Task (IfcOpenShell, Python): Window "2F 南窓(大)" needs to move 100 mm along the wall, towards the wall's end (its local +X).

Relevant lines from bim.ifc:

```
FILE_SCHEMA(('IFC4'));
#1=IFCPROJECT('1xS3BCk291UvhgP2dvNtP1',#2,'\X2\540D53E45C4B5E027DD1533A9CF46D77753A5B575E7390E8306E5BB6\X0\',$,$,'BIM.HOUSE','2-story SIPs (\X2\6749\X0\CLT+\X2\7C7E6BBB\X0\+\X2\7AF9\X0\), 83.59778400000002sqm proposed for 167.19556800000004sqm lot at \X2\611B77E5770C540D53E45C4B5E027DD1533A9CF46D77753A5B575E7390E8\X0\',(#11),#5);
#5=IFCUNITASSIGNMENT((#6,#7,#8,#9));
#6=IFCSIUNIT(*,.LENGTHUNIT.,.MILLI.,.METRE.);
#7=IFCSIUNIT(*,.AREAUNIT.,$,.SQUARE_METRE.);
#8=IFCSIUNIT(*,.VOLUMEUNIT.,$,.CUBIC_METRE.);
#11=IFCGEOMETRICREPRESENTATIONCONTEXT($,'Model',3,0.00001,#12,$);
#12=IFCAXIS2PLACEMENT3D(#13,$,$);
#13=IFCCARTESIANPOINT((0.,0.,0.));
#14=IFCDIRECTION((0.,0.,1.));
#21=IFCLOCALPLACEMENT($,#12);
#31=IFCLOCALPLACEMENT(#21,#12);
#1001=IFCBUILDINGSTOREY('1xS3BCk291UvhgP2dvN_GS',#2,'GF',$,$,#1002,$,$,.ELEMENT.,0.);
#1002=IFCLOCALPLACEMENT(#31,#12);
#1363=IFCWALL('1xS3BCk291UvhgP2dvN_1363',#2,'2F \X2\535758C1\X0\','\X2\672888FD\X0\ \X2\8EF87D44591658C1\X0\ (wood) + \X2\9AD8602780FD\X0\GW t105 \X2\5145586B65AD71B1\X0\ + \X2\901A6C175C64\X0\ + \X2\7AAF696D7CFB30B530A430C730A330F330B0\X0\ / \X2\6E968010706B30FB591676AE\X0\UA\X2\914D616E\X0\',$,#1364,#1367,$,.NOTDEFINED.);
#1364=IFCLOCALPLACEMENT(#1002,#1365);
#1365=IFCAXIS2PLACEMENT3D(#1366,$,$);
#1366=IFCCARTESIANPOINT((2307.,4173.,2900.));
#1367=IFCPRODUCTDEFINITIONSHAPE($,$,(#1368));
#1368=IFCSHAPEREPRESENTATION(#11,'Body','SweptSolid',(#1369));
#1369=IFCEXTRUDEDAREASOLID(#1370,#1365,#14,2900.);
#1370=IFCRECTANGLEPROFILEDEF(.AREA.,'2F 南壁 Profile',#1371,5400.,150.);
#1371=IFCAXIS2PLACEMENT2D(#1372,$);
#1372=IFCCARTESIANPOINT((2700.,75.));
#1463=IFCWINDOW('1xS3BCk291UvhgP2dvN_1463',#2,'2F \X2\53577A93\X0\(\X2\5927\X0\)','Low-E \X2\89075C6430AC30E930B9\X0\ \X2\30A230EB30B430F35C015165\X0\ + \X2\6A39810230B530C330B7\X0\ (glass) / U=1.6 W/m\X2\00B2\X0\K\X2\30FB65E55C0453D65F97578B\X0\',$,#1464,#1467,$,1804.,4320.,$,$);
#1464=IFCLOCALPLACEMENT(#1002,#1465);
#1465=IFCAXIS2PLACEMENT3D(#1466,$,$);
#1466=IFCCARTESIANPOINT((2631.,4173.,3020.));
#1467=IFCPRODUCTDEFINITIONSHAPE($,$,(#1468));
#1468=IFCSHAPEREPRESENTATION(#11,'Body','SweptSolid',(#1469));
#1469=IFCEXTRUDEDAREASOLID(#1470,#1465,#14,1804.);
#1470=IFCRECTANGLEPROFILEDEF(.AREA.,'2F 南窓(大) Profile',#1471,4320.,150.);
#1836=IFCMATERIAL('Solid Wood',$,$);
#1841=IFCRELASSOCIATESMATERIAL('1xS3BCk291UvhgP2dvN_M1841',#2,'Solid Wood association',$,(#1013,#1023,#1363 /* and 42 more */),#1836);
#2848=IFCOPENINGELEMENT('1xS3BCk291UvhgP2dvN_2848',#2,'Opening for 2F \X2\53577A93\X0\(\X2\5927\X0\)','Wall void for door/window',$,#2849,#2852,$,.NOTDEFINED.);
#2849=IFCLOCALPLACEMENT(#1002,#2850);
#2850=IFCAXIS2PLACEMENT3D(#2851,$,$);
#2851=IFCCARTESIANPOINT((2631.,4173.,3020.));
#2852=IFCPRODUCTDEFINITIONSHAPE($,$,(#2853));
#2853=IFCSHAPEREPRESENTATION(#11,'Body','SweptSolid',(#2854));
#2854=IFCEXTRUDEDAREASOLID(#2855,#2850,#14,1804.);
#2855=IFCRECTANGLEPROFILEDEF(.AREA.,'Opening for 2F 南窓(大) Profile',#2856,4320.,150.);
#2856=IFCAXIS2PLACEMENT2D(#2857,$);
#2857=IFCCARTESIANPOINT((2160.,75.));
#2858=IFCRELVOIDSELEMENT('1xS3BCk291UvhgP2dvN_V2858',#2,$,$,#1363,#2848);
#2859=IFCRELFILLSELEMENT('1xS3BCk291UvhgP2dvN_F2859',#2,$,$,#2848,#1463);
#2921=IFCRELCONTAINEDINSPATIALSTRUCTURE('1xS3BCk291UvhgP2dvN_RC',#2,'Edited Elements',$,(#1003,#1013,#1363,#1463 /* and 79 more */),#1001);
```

```python
import ifcopenshell
import ifcopenshell.api.geometry
import ifcopenshell.util.placement
import ifcopenshell.util.unit

model = ifcopenshell.open("bim.ifc")
unit_scale = ifcopenshell.util.unit.calculate_unit_scale(model)

window = model.by_guid("1xS3BCk291UvhgP2dvN_1463")
opening = window.FillsVoids[0].RelatingOpeningElement
wall = opening.VoidsElements[0].RelatingBuildingElement

wall_matrix = ifcopenshell.util.placement.get_local_placement(wall.ObjectPlacement)
shift = wall_matrix[:3, 0] * 0.1 / unit_scale
before = ifcopenshell.util.placement.get_local_placement(window.ObjectPlacement)[:3, 3].copy()

# The window is not placed relative to its opening, so move both.
for product in (opening, window):
    matrix = ifcopenshell.util.placement.get_local_placement(product.ObjectPlacement)
    matrix[:3, 3] += shift
    ifcopenshell.api.geometry.edit_object_placement(model, product=product, matrix=matrix, is_si=False)

after = ifcopenshell.util.placement.get_local_placement(window.ObjectPlacement)[:3, 3]
print("window moved by", (after - before).round(3) + 0.0)

model.write("bim_edited.ifc")
```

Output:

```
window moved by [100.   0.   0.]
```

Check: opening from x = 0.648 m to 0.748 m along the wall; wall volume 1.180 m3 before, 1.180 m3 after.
